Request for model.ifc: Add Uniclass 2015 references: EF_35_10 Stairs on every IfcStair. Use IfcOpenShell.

First a look at what the model holds.

```python
import ifcopenshell

model = ifcopenshell.open("model.ifc")
print(model.schema)
print("classifications:", [c.Name for c in model.by_type("IfcClassification")])
for ifc_class in ("IfcDoor", "IfcRoof", "IfcStair", "IfcWall", "IfcWindow"):
    print(ifc_class, len(model.by_type(ifc_class)))
```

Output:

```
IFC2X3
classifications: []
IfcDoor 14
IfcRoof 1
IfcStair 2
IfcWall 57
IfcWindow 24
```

```python
import ifcopenshell
import ifcopenshell.api.classification

model = ifcopenshell.open("model.ifc")

# IFC2X3 requires Source and Edition and has no link from the project to the system.
system = model.create_entity("IfcClassification", Source="NBS", Edition="2015", Name="Uniclass 2015")

codes = {
    "IfcStair": ("EF_35_10", "Stairs"),
}
for ifc_class, (code, name) in codes.items():
    products = model.by_type(ifc_class)
    ifcopenshell.api.classification.add_reference(
        model, products=products, classification=system, identification=code, name=name
    )
    print(code, len(products))

model.write("model_rev.ifc")
```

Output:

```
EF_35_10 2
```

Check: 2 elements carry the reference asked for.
